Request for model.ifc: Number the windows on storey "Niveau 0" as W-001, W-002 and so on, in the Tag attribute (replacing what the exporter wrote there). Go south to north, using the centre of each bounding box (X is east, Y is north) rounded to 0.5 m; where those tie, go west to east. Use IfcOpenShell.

First a look at what the model holds.

```python
import ifcopenshell
import ifcopenshell.util.element
import ifcopenshell.util.placement

model = ifcopenshell.open("model.ifc")
print(model.schema)
storey = next(s for s in model.by_type("IfcBuildingStorey") if s.Name == "Niveau 0")
windows = [e for e in ifcopenshell.util.element.get_decomposition(storey) if e.is_a("IfcWindow")]
for e in sorted(windows, key=lambda e: e.id()):
    origin = ifcopenshell.util.placement.get_local_placement(e.ObjectPlacement)[:3, 3]
    print(e.id(), e.Tag, e.Name, origin.round(2) + 0.0, sep=" | ")
```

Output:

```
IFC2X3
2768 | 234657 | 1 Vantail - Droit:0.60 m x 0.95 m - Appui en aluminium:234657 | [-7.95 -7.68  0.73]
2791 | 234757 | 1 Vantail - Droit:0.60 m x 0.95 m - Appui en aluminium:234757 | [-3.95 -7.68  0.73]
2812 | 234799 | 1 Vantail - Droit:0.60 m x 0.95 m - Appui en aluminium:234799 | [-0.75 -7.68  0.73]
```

```python
import ifcopenshell
import ifcopenshell.geom
import ifcopenshell.util.element
import ifcopenshell.util.shape

model = ifcopenshell.open("model.ifc")
settings = ifcopenshell.geom.settings()
settings.set("use-world-coords", True)


def centre(element):
    shape = ifcopenshell.geom.create_shape(settings, element)
    return ifcopenshell.util.shape.get_bbox_centroid(shape.geometry)


storey = next(s for s in model.by_type("IfcBuildingStorey") if s.Name == "Niveau 0")
windows = [e for e in ifcopenshell.util.element.get_decomposition(storey) if e.is_a("IfcWindow")]

# Insertion points can sit at a corner or the storey origin, so sort by the geometry (in metres).
centres = {e: centre(e) for e in windows}
windows.sort(key=lambda e: (round(centres[e][1] / 0.5), centres[e][0]))

for i, e in enumerate(windows, start=1):
    number = f"W-0{i:02d}"
    e.Tag = number
    print(e.id(), number)

model.write("model_v2.ifc")
```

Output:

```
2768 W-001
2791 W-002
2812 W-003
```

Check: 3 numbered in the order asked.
